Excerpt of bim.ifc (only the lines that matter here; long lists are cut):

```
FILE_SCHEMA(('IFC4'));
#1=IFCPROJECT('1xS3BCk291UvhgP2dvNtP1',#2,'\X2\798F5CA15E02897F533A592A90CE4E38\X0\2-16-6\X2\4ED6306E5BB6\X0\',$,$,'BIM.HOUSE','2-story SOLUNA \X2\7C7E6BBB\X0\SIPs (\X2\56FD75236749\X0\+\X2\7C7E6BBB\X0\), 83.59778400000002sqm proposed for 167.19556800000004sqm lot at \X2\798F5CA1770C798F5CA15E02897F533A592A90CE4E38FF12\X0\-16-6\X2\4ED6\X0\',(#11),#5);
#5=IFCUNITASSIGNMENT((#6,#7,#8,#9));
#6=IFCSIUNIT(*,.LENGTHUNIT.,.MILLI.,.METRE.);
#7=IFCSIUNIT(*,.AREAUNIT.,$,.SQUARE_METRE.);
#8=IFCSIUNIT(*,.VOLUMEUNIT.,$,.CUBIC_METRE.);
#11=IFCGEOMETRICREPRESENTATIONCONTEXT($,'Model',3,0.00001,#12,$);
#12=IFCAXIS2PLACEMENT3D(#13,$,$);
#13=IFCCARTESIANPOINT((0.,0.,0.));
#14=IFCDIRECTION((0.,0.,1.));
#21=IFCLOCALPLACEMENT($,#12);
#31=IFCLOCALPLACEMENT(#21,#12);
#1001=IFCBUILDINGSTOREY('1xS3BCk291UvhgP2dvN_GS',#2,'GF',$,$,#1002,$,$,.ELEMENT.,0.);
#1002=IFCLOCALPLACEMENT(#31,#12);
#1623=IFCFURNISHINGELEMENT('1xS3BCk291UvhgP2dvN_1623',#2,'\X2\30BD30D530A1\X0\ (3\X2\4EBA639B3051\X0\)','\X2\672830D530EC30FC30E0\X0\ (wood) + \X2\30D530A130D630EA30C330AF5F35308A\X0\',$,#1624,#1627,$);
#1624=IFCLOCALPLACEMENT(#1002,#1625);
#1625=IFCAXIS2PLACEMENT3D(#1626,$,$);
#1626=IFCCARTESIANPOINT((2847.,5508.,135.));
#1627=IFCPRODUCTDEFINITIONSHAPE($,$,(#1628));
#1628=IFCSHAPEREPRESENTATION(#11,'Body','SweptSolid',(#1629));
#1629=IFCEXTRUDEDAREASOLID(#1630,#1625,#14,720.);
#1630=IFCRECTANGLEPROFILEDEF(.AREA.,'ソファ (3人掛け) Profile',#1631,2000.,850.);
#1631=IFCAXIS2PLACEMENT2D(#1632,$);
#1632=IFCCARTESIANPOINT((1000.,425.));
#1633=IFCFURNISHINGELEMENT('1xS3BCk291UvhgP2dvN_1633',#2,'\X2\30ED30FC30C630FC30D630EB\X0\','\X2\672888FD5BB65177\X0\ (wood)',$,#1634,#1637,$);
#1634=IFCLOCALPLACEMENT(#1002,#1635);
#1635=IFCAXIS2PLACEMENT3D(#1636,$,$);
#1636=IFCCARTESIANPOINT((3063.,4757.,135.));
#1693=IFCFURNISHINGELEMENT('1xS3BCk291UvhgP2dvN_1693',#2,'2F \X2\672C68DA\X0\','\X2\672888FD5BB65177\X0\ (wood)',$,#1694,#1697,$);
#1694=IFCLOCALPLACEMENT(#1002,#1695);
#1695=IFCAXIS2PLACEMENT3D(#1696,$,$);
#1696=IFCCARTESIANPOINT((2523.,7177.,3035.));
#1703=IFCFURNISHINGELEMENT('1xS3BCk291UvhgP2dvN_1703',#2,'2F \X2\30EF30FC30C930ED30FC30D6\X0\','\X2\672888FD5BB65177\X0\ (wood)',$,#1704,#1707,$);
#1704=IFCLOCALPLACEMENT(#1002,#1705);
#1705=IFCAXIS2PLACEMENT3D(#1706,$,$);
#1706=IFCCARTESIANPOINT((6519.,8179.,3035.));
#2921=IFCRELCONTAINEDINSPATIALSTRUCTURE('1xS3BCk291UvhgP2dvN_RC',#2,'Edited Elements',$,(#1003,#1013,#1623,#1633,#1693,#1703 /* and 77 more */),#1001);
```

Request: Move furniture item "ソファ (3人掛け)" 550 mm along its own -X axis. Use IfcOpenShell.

```python
import ifcopenshell
import ifcopenshell.api.geometry
import ifcopenshell.util.placement

model = ifcopenshell.open("bim.ifc")

item = model.by_guid("1xS3BCk291UvhgP2dvN_1623")
matrix = ifcopenshell.util.placement.get_local_placement(item.ObjectPlacement)
matrix[:3, 3] -= matrix[:3, 0] * 550.0
ifcopenshell.api.geometry.edit_object_placement(model, product=item, matrix=matrix, is_si=False)

print(ifcopenshell.util.placement.get_local_placement(item.ObjectPlacement).round(3) + 0.0)

model.write("bim_edited.ifc")
```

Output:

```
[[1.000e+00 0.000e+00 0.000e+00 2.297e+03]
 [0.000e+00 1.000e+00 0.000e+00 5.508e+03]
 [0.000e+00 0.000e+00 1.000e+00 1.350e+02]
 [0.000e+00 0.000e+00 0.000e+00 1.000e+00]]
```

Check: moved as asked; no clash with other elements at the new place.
